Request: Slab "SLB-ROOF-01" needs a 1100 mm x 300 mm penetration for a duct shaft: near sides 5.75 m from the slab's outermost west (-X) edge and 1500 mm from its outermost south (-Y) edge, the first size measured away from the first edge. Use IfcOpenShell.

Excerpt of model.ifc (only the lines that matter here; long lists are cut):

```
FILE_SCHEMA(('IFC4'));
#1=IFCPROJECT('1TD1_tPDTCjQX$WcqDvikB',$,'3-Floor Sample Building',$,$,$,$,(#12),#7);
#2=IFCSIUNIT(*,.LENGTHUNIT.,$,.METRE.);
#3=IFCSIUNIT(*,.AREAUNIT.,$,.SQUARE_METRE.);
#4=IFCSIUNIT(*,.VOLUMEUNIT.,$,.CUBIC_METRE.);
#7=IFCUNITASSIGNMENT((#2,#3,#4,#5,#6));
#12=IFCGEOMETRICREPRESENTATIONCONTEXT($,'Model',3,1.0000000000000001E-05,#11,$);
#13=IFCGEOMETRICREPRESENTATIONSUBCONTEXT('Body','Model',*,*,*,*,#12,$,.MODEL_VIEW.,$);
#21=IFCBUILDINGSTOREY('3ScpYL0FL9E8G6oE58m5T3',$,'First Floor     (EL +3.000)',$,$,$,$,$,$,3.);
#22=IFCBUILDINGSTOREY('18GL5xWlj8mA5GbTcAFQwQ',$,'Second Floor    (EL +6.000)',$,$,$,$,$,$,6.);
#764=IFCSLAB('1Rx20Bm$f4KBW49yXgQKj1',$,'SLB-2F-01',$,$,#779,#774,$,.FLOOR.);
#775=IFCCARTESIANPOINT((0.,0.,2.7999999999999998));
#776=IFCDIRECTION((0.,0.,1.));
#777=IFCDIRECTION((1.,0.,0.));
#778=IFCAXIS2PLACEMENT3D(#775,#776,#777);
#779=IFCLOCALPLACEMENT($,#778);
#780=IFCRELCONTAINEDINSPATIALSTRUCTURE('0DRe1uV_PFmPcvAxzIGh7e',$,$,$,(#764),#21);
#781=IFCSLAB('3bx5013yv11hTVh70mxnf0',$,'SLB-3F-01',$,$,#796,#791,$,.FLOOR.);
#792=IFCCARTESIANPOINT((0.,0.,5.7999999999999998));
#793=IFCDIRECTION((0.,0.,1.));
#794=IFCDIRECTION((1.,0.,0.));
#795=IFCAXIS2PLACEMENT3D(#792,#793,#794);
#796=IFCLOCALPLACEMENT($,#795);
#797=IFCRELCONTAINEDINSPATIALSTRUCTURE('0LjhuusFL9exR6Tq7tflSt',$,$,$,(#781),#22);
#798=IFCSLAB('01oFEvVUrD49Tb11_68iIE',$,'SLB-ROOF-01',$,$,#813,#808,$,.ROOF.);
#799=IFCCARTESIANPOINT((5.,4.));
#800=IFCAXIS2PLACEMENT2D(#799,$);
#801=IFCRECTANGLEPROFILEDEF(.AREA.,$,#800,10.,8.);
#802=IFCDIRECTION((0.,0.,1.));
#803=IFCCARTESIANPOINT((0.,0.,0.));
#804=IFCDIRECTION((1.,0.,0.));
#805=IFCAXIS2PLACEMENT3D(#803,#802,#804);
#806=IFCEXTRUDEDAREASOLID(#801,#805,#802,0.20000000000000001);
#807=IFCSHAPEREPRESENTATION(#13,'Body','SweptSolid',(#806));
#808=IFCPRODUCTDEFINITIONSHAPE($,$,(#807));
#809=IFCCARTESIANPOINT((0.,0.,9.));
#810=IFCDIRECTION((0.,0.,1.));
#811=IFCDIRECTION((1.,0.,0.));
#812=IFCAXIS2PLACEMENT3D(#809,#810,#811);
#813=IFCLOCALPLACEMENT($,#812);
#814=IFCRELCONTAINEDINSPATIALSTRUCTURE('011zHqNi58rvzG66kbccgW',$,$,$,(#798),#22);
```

```python
import numpy as np
import ifcopenshell
import ifcopenshell.api.feature
import ifcopenshell.api.geometry
import ifcopenshell.api.root
import ifcopenshell.geom
import ifcopenshell.util.placement
import ifcopenshell.util.representation
import ifcopenshell.util.shape
import ifcopenshell.util.unit

model = ifcopenshell.open("model.ifc")
unit_scale = ifcopenshell.util.unit.calculate_unit_scale(model)
settings = ifcopenshell.geom.settings()


def volume(element):
    """Net volume in cubic metres, openings subtracted."""
    shape = ifcopenshell.geom.create_shape(settings, element)
    return ifcopenshell.util.shape.get_volume(shape.geometry)


slab = model.by_id(798)
before = volume(slab)

# Extent in the slab's own axes, in metres. The edges named are its -X and -Y sides.
slab_shape = ifcopenshell.geom.create_shape(settings, slab)
vertices = ifcopenshell.util.shape.get_vertices(slab_shape.geometry)
x_min, y_min, bottom = vertices.min(axis=0)
top = vertices[:, 2].max()

opening = ifcopenshell.api.root.create_entity(model, ifc_class="IfcOpeningElement", name="Duct shaft opening", predefined_type="OPENING")
context = ifcopenshell.util.representation.get_context(model, "Model", "Body", "MODEL_VIEW")
width, depth = 1.1, 0.3
outline = [(0.0, 0.0), (width, 0.0), (width, depth), (0.0, depth), (0.0, 0.0)]
# Overshoot both faces by 50 mm so the cut is clean.
shape = ifcopenshell.api.geometry.add_slab_representation(
    model, context=context, depth=top - bottom + 0.1, polyline=outline
)
ifcopenshell.api.geometry.assign_representation(model, product=opening, representation=shape)

matrix = ifcopenshell.util.placement.get_local_placement(slab.ObjectPlacement)
matrix[:, 3] = matrix @ np.append(np.array([x_min + 5.75, y_min + 1.5, bottom - 0.05]) / unit_scale, 1.0)
ifcopenshell.api.geometry.edit_object_placement(model, product=opening, matrix=matrix, is_si=False)
ifcopenshell.api.feature.add_feature(model, feature=opening, element=slab)

after = volume(slab)

print(f"slab volume {before:.3f} -> {after:.3f} m3")

model.write("model_rev.ifc")
```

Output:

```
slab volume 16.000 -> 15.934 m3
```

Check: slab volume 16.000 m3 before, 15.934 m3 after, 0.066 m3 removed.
